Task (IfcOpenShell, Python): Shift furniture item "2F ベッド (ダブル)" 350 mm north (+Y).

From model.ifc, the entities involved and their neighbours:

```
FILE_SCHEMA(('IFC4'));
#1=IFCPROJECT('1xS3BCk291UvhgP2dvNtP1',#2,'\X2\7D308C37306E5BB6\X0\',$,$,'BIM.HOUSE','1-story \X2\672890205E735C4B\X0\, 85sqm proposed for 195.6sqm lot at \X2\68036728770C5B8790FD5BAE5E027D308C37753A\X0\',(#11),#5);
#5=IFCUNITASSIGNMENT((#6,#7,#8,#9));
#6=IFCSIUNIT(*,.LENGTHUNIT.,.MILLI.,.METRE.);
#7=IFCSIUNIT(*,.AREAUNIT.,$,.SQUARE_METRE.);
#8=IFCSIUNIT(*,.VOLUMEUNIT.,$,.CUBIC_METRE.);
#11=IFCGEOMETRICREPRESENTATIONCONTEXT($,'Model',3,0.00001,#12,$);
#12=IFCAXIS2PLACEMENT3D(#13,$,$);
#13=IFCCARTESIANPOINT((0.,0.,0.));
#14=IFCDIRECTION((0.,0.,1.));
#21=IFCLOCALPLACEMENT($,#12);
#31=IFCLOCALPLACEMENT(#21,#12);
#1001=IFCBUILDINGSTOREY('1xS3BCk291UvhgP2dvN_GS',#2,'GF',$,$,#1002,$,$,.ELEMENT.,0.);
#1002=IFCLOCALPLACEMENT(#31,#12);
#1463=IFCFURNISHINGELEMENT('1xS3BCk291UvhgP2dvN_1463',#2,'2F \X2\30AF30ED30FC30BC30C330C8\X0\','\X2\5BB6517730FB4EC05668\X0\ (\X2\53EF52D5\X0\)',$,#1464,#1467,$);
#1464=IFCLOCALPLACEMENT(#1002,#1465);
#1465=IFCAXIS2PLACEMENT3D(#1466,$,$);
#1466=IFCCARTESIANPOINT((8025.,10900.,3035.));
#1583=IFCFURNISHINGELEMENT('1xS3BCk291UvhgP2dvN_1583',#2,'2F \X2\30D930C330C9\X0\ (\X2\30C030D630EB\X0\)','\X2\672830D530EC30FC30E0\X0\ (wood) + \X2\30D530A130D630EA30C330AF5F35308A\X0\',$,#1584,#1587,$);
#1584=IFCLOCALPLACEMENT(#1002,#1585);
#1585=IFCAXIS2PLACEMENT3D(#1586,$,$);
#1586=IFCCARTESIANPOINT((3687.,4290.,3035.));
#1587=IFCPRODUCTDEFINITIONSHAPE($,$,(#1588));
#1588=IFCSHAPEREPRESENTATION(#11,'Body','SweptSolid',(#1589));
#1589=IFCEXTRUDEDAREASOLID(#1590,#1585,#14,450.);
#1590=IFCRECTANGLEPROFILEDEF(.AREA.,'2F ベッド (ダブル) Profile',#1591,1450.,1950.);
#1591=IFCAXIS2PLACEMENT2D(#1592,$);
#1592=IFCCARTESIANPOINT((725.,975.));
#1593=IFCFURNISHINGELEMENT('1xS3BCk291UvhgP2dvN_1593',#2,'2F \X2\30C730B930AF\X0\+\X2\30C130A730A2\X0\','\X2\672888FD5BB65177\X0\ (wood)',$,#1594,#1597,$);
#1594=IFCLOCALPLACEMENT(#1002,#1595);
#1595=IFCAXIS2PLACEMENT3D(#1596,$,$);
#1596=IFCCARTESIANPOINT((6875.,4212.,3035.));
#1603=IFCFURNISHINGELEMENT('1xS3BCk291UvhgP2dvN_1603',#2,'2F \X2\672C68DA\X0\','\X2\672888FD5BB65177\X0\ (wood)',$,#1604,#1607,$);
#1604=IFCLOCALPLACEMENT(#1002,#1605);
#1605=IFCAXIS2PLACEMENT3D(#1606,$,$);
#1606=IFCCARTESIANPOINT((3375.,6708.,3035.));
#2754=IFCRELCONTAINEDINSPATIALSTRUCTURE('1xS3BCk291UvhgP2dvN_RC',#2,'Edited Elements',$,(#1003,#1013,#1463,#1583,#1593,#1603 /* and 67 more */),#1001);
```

```python
import ifcopenshell
import ifcopenshell.api.geometry
import ifcopenshell.util.placement

model = ifcopenshell.open("model.ifc")

item = model.by_id(1583)
matrix = ifcopenshell.util.placement.get_local_placement(item.ObjectPlacement)
matrix[1, 3] += 350.0
ifcopenshell.api.geometry.edit_object_placement(model, product=item, matrix=matrix, is_si=False)

print(ifcopenshell.util.placement.get_local_placement(item.ObjectPlacement).round(3) + 0.0)

model.write("model_updated.ifc")
```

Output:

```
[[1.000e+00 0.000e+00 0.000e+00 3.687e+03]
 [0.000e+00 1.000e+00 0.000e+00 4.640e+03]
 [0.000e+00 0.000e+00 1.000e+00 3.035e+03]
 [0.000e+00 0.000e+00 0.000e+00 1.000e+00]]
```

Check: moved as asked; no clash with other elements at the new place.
